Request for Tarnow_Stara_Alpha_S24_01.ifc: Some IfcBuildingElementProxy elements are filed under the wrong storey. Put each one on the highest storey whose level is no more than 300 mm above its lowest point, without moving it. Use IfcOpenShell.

First a look at what the model holds.

```python
import ifcopenshell
import ifcopenshell.util.element
import ifcopenshell.util.placement

model = ifcopenshell.open("Tarnow_Stara_Alpha_S24_01.ifc")
print(model.schema)
for storey in model.by_type("IfcBuildingStorey"):
    level = ifcopenshell.util.placement.get_storey_elevation(storey)
    count = sum(e.is_a("IfcBuildingElementProxy") for e in ifcopenshell.util.element.get_contained(storey))
    print(storey.id(), storey.Name, round(level, 3), count, sep=" | ")
```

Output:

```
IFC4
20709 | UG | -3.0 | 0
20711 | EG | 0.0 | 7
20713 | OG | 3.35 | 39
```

```python
import ifcopenshell
import ifcopenshell.api.spatial
import ifcopenshell.geom
import ifcopenshell.util.element
import ifcopenshell.util.placement
import ifcopenshell.util.shape
import ifcopenshell.util.unit

model = ifcopenshell.open("Tarnow_Stara_Alpha_S24_01.ifc")
unit_scale = ifcopenshell.util.unit.calculate_unit_scale(model)
settings = ifcopenshell.geom.settings()

levels = sorted(
    ((ifcopenshell.util.placement.get_storey_elevation(s) * unit_scale, s) for s in model.by_type("IfcBuildingStorey")),
    key=lambda pair: pair[0],
)

for e in model.by_type("IfcBuildingElementProxy"):
    current = e.ContainedInStructure[0].RelatingStructure if e.ContainedInStructure else None
    if current is None or not current.is_a("IfcBuildingStorey"):
        continue
    shape = ifcopenshell.geom.create_shape(settings, e)
    bottom = ifcopenshell.util.shape.get_shape_bottom_elevation(shape, shape.geometry)
    below = [s for level, s in levels if level <= bottom + 0.3]
    storey = below[-1] if below else levels[0][1]
    if storey != current:
        # assign_container keeps the world position.
        ifcopenshell.api.spatial.assign_container(model, products=[e], relating_structure=storey)
        print(e.id(), current.Name, "->", storey.Name)

model.write("Tarnow_Stara_Alpha_S24_01_rev.ifc")
```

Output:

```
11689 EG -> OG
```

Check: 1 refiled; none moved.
